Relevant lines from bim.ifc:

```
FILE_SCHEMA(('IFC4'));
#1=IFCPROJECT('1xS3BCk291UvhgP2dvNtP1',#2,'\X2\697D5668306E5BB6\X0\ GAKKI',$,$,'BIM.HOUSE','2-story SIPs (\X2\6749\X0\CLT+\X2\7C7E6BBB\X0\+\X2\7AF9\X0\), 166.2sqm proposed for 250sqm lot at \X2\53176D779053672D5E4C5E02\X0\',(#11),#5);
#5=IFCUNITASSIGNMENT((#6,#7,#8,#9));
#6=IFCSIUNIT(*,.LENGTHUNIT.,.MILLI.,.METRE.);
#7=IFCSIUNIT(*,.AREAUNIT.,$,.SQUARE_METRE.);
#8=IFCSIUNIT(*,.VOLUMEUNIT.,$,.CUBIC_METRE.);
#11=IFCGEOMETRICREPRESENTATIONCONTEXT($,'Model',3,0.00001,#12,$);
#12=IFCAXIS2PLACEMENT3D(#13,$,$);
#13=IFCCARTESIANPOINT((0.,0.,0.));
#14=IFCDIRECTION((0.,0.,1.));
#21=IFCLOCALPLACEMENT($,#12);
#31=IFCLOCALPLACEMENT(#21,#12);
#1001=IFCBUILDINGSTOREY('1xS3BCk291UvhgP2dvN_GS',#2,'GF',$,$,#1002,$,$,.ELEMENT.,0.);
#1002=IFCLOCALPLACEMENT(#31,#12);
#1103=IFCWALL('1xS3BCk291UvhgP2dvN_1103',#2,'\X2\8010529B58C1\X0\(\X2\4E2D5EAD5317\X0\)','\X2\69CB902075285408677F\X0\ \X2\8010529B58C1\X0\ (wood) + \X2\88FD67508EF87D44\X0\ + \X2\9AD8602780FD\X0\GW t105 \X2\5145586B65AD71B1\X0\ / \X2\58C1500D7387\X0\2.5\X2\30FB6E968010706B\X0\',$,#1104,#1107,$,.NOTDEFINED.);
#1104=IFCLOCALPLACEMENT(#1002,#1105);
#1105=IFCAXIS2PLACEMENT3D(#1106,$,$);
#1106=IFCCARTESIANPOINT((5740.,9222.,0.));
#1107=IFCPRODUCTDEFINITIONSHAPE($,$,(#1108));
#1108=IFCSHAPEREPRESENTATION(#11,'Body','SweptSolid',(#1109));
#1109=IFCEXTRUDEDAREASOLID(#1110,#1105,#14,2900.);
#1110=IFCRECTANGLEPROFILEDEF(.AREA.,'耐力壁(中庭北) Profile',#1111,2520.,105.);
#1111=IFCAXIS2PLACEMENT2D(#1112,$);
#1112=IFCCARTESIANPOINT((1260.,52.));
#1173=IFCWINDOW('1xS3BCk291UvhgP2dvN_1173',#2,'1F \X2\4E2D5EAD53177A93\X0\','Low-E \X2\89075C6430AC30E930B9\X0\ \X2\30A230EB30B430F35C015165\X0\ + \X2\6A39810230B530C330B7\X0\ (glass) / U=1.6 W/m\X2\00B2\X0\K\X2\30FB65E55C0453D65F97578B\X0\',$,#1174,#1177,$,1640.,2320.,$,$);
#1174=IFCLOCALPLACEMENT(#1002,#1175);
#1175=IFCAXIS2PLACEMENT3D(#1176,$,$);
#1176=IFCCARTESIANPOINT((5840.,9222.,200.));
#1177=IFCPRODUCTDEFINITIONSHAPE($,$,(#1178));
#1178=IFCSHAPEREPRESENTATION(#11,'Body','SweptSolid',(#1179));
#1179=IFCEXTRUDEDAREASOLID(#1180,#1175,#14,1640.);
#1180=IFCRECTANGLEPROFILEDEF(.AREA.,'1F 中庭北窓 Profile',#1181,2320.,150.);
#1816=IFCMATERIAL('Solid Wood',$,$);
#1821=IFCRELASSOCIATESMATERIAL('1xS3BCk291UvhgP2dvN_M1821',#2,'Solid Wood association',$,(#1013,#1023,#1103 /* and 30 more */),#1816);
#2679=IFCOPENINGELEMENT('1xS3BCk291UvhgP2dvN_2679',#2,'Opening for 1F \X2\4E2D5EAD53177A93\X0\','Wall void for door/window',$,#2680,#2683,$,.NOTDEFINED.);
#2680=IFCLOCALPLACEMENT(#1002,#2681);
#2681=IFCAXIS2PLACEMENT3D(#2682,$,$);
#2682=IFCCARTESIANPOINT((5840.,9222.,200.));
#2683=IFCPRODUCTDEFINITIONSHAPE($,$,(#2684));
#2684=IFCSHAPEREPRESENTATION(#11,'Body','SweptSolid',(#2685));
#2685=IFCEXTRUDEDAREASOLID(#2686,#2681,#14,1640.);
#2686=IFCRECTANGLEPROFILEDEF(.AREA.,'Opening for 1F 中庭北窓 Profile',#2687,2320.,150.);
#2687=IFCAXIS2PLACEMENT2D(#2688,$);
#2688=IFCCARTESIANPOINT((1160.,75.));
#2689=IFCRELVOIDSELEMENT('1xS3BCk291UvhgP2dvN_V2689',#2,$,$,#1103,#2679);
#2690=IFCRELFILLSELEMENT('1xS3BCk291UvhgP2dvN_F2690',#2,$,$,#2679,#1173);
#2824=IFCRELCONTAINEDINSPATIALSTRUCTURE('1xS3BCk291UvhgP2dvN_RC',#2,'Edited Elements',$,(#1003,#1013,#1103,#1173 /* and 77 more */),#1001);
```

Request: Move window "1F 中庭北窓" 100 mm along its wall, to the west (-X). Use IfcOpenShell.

```python
import ifcopenshell
import ifcopenshell.api.geometry
import ifcopenshell.util.placement
import ifcopenshell.util.unit

model = ifcopenshell.open("bim.ifc")
unit_scale = ifcopenshell.util.unit.calculate_unit_scale(model)

window = model.by_id(1173)
opening = window.FillsVoids[0].RelatingOpeningElement
wall = opening.VoidsElements[0].RelatingBuildingElement

wall_matrix = ifcopenshell.util.placement.get_local_placement(wall.ObjectPlacement)
shift = wall_matrix[:3, 0] * -0.1 / unit_scale
before = ifcopenshell.util.placement.get_local_placement(window.ObjectPlacement)[:3, 3].copy()

# The window is not placed relative to its opening, so move both.
for product in (opening, window):
    matrix = ifcopenshell.util.placement.get_local_placement(product.ObjectPlacement)
    matrix[:3, 3] += shift
    ifcopenshell.api.geometry.edit_object_placement(model, product=product, matrix=matrix, is_si=False)

after = ifcopenshell.util.placement.get_local_placement(window.ObjectPlacement)[:3, 3]
print("window moved by", (after - before).round(3) + 0.0)

model.write("bim_updated.ifc")
```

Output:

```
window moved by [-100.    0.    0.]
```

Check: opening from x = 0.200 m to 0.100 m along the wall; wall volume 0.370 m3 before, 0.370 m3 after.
